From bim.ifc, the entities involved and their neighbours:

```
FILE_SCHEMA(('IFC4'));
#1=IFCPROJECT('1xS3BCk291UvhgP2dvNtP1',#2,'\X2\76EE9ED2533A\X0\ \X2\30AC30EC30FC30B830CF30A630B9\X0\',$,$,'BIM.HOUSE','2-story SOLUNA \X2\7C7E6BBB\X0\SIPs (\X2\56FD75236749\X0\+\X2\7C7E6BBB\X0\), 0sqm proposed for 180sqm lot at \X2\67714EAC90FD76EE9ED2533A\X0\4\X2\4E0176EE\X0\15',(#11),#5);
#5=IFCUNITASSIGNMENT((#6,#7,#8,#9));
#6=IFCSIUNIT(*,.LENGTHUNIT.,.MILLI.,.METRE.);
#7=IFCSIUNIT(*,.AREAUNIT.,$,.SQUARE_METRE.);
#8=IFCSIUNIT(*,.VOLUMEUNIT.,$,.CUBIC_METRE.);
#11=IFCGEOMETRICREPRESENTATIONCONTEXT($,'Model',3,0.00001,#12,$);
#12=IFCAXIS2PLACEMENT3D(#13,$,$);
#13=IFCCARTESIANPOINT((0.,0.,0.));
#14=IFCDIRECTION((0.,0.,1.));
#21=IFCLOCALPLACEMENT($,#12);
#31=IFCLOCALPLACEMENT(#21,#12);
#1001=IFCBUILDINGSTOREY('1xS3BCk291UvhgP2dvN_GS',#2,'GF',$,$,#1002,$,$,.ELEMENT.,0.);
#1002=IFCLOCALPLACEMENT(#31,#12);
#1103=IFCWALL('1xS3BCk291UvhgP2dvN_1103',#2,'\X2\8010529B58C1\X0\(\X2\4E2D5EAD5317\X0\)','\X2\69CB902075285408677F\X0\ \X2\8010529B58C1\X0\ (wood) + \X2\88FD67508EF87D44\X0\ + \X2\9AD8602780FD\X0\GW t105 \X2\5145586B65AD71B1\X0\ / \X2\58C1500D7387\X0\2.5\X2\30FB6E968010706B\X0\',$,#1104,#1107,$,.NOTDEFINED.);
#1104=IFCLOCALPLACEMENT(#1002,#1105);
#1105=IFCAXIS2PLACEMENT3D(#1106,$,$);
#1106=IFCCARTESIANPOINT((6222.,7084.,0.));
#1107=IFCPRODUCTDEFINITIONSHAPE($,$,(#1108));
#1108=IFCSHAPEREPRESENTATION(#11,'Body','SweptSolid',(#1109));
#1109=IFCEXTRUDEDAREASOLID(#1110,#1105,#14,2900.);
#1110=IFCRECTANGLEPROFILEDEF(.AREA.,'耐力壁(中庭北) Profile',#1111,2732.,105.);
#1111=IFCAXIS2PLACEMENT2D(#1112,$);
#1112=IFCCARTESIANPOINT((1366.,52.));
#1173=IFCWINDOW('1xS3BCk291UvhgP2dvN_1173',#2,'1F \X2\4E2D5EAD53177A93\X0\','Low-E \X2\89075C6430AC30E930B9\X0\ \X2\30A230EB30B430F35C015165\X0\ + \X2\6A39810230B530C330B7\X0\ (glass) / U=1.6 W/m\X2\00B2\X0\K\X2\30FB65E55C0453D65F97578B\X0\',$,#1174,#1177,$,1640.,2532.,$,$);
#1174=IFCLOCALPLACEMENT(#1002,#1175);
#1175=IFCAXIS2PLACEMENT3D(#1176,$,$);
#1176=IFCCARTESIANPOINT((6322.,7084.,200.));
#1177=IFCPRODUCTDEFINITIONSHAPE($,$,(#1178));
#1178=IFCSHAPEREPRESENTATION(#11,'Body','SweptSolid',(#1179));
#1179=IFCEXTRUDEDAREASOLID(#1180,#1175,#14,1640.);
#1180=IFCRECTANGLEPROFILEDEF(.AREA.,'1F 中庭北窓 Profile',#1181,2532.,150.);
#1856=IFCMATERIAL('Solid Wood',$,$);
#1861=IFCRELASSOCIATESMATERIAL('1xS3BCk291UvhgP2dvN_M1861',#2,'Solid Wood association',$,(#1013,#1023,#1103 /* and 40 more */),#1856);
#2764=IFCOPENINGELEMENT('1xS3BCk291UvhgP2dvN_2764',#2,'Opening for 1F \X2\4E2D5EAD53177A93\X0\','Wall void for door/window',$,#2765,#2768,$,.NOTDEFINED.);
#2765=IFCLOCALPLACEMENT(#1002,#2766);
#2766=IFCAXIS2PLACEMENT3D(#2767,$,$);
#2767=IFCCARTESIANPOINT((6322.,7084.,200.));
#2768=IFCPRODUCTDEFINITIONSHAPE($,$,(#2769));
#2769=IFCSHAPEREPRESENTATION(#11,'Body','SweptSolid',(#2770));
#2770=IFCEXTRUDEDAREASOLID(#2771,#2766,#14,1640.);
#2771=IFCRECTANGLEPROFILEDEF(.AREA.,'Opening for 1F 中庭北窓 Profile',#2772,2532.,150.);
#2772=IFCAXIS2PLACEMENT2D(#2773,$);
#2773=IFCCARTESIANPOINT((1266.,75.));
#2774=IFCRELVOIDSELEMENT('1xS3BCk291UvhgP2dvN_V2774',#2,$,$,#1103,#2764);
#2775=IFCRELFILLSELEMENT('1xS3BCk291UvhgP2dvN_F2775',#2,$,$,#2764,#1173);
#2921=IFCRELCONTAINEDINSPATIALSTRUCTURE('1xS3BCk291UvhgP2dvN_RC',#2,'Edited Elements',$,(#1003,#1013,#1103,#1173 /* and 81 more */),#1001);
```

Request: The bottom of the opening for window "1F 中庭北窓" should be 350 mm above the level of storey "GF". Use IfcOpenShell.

```python
import numpy as np
import ifcopenshell
import ifcopenshell.api.geometry
import ifcopenshell.geom
import ifcopenshell.util.element
import ifcopenshell.util.placement
import ifcopenshell.util.shape
import ifcopenshell.util.unit

model = ifcopenshell.open("bim.ifc")
unit_scale = ifcopenshell.util.unit.calculate_unit_scale(model)

window = model.by_guid("1xS3BCk291UvhgP2dvN_1173")
opening = window.FillsVoids[0].RelatingOpeningElement
storey = ifcopenshell.util.element.get_container(window, ifc_class="IfcBuildingStorey")
level = ifcopenshell.util.placement.get_local_placement(storey.ObjectPlacement)[2, 3]

# The opening's origin need not be at the sill, so measure its lowest point.
shape = ifcopenshell.geom.create_shape(ifcopenshell.geom.settings(), opening)
bottom = ifcopenshell.util.shape.get_shape_bottom_elevation(shape, shape.geometry) / unit_scale
dz = level + 0.35 / unit_scale - bottom

shift = np.array([0.0, 0.0, dz])
# The window is not placed relative to its opening, so move both.
for product in (opening, window):
    matrix = ifcopenshell.util.placement.get_local_placement(product.ObjectPlacement)
    matrix[:3, 3] += shift
    ifcopenshell.api.geometry.edit_object_placement(model, product=product, matrix=matrix, is_si=False)

print(f"moved by {dz * unit_scale:+.3f} m")

model.write("bim_edited.ifc")
```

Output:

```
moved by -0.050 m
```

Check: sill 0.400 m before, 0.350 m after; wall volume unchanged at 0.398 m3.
